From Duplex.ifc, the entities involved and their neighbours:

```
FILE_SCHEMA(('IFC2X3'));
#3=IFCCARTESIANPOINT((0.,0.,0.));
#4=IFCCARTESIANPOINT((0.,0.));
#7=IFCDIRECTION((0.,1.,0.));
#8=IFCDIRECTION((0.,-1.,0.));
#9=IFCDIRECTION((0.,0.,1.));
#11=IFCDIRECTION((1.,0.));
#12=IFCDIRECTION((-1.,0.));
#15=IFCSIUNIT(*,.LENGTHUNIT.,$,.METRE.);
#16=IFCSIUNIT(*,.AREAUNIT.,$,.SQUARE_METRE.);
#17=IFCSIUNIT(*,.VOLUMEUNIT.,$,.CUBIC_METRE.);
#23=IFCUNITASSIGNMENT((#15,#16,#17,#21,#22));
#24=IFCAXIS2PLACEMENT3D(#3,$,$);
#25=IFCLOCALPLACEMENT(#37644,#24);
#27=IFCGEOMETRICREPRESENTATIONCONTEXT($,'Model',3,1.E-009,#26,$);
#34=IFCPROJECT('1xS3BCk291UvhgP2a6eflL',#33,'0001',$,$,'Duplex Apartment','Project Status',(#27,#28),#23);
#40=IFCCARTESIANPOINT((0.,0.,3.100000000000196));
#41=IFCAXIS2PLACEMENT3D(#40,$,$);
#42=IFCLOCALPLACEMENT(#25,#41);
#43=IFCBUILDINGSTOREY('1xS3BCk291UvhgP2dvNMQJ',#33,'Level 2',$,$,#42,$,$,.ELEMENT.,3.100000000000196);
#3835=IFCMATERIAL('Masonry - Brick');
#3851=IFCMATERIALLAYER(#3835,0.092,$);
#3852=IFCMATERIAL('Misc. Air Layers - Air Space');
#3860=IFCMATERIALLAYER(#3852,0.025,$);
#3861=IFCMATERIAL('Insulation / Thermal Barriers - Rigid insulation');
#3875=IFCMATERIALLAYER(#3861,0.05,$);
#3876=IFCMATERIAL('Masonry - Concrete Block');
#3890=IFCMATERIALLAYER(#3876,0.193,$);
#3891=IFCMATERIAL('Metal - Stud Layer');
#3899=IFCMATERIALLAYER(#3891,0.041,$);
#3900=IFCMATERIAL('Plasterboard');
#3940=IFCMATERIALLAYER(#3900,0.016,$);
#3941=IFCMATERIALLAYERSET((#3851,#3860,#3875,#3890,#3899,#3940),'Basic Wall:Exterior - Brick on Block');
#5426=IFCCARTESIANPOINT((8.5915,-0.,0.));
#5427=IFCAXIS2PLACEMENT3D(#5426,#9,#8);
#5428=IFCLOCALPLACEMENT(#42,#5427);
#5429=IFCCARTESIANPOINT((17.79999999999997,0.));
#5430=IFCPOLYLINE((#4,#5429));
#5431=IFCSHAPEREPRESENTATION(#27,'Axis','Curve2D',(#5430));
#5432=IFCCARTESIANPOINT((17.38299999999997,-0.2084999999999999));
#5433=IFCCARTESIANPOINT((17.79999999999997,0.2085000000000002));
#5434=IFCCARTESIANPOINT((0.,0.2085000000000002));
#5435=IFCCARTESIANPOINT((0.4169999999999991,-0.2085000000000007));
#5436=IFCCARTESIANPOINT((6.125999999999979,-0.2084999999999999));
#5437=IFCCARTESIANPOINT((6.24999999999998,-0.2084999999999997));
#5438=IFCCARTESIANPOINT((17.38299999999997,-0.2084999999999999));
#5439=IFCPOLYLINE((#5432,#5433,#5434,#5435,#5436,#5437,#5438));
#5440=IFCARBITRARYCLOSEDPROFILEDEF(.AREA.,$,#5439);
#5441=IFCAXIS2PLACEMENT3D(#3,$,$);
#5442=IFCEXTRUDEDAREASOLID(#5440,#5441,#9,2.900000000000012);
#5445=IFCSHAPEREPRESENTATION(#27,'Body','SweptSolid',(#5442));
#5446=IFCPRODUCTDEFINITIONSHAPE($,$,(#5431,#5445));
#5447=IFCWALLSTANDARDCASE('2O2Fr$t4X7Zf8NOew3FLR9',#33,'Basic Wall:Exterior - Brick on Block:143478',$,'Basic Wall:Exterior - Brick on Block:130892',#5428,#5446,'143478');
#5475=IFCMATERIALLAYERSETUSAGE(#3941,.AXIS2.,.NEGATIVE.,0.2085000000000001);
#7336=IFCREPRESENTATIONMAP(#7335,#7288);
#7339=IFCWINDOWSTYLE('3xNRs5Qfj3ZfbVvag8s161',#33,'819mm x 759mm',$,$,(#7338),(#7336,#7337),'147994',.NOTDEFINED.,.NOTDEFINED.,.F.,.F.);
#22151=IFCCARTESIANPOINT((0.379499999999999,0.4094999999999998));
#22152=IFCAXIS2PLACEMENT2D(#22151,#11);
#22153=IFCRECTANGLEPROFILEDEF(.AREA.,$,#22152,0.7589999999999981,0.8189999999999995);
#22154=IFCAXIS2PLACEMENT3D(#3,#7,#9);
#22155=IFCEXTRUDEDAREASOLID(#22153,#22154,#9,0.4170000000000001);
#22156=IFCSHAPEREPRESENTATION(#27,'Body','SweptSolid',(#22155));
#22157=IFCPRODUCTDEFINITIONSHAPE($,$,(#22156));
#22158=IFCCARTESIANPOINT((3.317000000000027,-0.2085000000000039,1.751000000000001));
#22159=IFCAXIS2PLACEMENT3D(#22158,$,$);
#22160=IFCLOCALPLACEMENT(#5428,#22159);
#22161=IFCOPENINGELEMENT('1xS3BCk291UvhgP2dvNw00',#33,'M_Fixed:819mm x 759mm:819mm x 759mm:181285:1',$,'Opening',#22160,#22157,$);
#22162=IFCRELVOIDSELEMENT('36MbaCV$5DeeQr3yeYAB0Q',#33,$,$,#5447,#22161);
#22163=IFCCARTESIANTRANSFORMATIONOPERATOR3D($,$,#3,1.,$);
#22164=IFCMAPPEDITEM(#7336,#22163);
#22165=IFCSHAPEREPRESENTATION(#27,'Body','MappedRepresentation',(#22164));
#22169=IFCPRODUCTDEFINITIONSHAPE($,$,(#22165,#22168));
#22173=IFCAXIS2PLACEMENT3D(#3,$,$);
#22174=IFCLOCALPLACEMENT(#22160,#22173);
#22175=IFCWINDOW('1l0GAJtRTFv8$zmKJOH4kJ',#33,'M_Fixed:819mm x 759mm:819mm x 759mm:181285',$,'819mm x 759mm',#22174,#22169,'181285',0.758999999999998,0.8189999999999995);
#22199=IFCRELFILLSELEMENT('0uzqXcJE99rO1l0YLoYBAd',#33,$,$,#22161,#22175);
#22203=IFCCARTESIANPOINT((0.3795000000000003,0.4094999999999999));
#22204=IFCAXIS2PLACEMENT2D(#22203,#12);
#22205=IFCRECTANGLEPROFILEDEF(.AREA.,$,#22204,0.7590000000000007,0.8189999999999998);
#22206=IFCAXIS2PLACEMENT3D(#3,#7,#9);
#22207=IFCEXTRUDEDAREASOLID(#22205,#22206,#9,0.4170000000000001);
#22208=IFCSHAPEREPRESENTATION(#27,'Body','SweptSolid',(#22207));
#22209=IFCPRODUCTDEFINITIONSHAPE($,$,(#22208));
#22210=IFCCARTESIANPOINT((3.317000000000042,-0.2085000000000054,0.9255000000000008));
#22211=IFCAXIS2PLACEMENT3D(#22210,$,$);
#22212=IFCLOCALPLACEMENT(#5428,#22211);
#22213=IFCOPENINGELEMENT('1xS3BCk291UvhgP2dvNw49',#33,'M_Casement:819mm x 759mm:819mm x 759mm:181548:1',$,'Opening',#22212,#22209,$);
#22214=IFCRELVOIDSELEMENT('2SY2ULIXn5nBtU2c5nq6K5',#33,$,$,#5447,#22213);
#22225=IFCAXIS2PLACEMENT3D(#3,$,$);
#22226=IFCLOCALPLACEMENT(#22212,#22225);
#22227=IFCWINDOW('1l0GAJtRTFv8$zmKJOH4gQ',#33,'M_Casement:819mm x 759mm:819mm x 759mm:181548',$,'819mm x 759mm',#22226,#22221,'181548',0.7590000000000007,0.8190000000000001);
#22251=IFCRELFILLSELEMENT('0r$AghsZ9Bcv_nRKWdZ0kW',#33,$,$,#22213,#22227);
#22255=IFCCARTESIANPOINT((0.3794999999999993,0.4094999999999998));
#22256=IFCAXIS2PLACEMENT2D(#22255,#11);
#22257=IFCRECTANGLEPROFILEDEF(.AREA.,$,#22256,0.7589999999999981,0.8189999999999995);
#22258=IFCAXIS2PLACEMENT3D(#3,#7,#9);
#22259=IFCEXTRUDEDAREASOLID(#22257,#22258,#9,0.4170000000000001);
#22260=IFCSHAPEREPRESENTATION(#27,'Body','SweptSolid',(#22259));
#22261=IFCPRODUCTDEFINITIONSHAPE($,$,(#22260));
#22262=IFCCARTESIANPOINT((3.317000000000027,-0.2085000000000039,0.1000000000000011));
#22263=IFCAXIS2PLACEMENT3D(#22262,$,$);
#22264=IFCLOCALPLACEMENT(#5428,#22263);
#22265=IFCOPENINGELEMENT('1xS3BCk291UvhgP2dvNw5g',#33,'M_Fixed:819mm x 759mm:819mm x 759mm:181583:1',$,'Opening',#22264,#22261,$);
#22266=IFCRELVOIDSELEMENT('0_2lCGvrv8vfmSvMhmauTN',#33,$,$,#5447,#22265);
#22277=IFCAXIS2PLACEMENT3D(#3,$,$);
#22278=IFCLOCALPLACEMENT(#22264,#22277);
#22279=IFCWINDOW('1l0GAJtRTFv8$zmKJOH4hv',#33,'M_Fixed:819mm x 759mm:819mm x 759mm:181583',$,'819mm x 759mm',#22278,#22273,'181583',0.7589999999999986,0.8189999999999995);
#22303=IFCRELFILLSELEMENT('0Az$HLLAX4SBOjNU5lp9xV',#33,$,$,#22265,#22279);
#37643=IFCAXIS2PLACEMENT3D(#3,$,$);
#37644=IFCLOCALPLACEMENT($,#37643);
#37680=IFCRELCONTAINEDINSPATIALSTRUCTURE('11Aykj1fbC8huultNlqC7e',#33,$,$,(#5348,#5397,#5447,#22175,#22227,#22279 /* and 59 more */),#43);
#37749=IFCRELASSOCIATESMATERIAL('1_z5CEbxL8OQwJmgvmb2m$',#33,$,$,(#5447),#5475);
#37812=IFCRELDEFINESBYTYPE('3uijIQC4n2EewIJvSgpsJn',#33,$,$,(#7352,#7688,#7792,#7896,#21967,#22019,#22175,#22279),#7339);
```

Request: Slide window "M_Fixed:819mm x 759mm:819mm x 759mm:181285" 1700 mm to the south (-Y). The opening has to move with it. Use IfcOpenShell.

```python
import ifcopenshell
import ifcopenshell.api.geometry
import ifcopenshell.util.placement
import ifcopenshell.util.unit

model = ifcopenshell.open("Duplex.ifc")
unit_scale = ifcopenshell.util.unit.calculate_unit_scale(model)

window = model.by_guid("1l0GAJtRTFv8$zmKJOH4kJ")
opening = window.FillsVoids[0].RelatingOpeningElement
wall = opening.VoidsElements[0].RelatingBuildingElement

wall_matrix = ifcopenshell.util.placement.get_local_placement(wall.ObjectPlacement)
shift = wall_matrix[:3, 0] * 1.7 / unit_scale
before = ifcopenshell.util.placement.get_local_placement(window.ObjectPlacement)[:3, 3].copy()

# The window is placed relative to its opening, so it follows when the opening moves.
matrix = ifcopenshell.util.placement.get_local_placement(opening.ObjectPlacement)
matrix[:3, 3] += shift
ifcopenshell.api.geometry.edit_object_placement(
    model, product=opening, matrix=matrix, is_si=False, should_transform_children=True
)

after = ifcopenshell.util.placement.get_local_placement(window.ObjectPlacement)[:3, 3]
print("window moved by", (after - before).round(3) + 0.0)

model.write("Duplex_edited.ifc")
```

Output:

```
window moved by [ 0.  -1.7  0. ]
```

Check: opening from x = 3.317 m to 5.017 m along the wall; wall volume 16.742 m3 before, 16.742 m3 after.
